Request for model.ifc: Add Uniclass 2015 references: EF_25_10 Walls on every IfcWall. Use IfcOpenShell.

First a look at what the model holds.

```python
import ifcopenshell

model = ifcopenshell.open("model.ifc")
print(model.schema)
print("classifications:", [c.Name for c in model.by_type("IfcClassification")])
for ifc_class in ("IfcDoor", "IfcRoof", "IfcStair", "IfcWall", "IfcWindow"):
    print(ifc_class, len(model.by_type(ifc_class)))
```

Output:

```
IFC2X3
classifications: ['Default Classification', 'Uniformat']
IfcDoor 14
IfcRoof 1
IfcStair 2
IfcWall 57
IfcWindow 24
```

```python
import ifcopenshell
import ifcopenshell.api.classification

model = ifcopenshell.open("model.ifc")

# IFC2X3 requires Source and Edition and has no link from the project to the system.
system = model.create_entity("IfcClassification", Source="NBS", Edition="2015", Name="Uniclass 2015")

codes = {
    "IfcWall": ("EF_25_10", "Walls"),
}
for ifc_class, (code, name) in codes.items():
    products = model.by_type(ifc_class)
    ifcopenshell.api.classification.add_reference(
        model, products=products, classification=system, identification=code, name=name
    )
    print(code, len(products))

model.write("model_v2.ifc")
```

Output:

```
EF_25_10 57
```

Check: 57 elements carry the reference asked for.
